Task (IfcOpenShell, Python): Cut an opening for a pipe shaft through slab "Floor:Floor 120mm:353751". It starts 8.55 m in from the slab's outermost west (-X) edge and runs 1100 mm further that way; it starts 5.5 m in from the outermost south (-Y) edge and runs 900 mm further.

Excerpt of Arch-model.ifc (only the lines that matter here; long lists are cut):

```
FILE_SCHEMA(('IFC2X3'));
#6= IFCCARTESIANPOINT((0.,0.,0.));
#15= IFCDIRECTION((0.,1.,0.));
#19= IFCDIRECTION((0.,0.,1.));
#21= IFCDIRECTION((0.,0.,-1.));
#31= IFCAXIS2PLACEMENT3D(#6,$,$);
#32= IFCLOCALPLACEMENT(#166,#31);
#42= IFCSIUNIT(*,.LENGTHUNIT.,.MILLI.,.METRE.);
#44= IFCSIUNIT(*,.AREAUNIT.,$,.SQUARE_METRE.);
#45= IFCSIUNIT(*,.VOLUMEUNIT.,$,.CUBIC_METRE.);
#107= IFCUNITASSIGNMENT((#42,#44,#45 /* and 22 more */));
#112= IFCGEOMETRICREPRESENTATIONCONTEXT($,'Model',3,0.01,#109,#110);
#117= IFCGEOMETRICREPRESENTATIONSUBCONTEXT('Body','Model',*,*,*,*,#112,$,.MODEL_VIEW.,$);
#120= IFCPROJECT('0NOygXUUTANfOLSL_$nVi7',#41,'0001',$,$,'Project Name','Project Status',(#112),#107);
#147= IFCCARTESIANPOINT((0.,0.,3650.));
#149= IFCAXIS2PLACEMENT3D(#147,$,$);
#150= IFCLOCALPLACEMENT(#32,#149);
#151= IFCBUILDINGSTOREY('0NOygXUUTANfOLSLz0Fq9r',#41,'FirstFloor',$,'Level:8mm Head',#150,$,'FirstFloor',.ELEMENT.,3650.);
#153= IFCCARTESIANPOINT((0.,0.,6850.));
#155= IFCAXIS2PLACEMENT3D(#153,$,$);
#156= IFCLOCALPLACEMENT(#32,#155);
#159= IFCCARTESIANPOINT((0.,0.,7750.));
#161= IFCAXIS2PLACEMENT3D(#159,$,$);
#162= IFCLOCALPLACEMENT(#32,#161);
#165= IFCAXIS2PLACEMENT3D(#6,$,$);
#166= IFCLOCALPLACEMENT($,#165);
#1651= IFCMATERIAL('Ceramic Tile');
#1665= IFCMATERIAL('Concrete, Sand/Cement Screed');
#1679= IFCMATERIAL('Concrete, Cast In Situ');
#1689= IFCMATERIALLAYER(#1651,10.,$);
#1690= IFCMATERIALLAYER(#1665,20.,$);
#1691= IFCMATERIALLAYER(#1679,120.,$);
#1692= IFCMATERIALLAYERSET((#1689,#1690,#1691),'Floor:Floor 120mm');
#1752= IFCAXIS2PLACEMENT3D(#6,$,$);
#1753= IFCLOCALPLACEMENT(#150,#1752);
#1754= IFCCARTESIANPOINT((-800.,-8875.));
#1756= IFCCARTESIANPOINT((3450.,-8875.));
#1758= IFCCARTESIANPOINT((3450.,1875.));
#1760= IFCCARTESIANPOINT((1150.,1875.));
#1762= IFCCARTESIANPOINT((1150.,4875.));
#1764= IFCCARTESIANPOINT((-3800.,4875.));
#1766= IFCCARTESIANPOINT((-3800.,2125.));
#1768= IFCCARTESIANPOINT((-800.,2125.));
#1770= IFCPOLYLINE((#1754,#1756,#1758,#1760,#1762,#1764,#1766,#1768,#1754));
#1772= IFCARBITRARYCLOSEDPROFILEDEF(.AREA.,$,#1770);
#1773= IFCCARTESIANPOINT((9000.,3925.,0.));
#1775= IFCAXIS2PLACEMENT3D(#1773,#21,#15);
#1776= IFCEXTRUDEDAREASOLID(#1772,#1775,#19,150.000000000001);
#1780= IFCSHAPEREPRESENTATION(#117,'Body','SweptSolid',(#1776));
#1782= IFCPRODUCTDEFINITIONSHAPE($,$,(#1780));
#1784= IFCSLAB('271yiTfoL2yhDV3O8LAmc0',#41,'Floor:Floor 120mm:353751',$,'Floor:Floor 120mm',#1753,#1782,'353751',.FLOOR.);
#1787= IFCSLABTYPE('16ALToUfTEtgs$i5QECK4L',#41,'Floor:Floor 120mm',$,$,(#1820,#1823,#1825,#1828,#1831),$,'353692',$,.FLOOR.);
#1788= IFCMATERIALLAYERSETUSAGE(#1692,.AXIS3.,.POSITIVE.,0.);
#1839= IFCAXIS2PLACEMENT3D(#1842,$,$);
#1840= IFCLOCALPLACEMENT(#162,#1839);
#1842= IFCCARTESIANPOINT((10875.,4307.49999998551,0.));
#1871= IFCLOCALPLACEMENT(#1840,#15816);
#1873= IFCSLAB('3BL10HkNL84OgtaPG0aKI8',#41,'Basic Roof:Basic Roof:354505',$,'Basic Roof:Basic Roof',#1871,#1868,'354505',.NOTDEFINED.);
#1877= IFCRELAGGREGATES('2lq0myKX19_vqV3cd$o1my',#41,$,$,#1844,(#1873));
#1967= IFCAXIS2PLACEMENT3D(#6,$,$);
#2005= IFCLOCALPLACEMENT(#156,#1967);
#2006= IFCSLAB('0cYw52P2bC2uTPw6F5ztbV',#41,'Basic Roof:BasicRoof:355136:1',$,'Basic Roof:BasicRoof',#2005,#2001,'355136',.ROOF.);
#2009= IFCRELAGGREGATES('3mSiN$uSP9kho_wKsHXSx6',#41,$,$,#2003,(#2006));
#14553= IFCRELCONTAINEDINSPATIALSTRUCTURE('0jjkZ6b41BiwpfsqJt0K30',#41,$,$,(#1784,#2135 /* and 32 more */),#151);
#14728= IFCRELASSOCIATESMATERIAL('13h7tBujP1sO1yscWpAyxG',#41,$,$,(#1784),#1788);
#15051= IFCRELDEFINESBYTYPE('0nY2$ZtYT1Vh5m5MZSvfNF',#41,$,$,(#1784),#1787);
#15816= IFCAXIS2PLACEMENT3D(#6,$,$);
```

```python
import numpy as np
import ifcopenshell
import ifcopenshell.api.feature
import ifcopenshell.api.geometry
import ifcopenshell.api.root
import ifcopenshell.geom
import ifcopenshell.util.placement
import ifcopenshell.util.representation
import ifcopenshell.util.shape
import ifcopenshell.util.unit

model = ifcopenshell.open("Arch-model.ifc")
unit_scale = ifcopenshell.util.unit.calculate_unit_scale(model)
settings = ifcopenshell.geom.settings()


def volume(element):
    """Net volume in cubic metres, openings subtracted."""
    shape = ifcopenshell.geom.create_shape(settings, element)
    return ifcopenshell.util.shape.get_volume(shape.geometry)


slab = model.by_guid("271yiTfoL2yhDV3O8LAmc0")
before = volume(slab)

# Extent in the slab's own axes, in metres. The edges named are its -X and -Y sides.
slab_shape = ifcopenshell.geom.create_shape(settings, slab)
vertices = ifcopenshell.util.shape.get_vertices(slab_shape.geometry)
x_min, y_min, bottom = vertices.min(axis=0)
top = vertices[:, 2].max()

opening = ifcopenshell.api.root.create_entity(model, ifc_class="IfcOpeningElement", name="Pipe shaft opening")
context = ifcopenshell.util.representation.get_context(model, "Model", "Body", "MODEL_VIEW")
width, depth = 1.1, 0.9
outline = [(0.0, 0.0), (width, 0.0), (width, depth), (0.0, depth), (0.0, 0.0)]
# Overshoot both faces by 50 mm so the cut is clean.
shape = ifcopenshell.api.geometry.add_slab_representation(
    model, context=context, depth=top - bottom + 0.1, polyline=outline
)
ifcopenshell.api.geometry.assign_representation(model, product=opening, representation=shape)

matrix = ifcopenshell.util.placement.get_local_placement(slab.ObjectPlacement)
matrix[:, 3] = matrix @ np.append(np.array([x_min + 8.55, y_min + 5.5, bottom - 0.05]) / unit_scale, 1.0)
ifcopenshell.api.geometry.edit_object_placement(model, product=opening, matrix=matrix, is_si=False)
ifcopenshell.api.feature.add_feature(model, feature=opening, element=slab)

after = volume(slab)

print(f"slab volume {before:.3f} -> {after:.3f} m3")

model.write("Arch-model-out.ifc")
```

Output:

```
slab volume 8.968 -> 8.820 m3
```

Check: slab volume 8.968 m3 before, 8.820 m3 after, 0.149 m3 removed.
